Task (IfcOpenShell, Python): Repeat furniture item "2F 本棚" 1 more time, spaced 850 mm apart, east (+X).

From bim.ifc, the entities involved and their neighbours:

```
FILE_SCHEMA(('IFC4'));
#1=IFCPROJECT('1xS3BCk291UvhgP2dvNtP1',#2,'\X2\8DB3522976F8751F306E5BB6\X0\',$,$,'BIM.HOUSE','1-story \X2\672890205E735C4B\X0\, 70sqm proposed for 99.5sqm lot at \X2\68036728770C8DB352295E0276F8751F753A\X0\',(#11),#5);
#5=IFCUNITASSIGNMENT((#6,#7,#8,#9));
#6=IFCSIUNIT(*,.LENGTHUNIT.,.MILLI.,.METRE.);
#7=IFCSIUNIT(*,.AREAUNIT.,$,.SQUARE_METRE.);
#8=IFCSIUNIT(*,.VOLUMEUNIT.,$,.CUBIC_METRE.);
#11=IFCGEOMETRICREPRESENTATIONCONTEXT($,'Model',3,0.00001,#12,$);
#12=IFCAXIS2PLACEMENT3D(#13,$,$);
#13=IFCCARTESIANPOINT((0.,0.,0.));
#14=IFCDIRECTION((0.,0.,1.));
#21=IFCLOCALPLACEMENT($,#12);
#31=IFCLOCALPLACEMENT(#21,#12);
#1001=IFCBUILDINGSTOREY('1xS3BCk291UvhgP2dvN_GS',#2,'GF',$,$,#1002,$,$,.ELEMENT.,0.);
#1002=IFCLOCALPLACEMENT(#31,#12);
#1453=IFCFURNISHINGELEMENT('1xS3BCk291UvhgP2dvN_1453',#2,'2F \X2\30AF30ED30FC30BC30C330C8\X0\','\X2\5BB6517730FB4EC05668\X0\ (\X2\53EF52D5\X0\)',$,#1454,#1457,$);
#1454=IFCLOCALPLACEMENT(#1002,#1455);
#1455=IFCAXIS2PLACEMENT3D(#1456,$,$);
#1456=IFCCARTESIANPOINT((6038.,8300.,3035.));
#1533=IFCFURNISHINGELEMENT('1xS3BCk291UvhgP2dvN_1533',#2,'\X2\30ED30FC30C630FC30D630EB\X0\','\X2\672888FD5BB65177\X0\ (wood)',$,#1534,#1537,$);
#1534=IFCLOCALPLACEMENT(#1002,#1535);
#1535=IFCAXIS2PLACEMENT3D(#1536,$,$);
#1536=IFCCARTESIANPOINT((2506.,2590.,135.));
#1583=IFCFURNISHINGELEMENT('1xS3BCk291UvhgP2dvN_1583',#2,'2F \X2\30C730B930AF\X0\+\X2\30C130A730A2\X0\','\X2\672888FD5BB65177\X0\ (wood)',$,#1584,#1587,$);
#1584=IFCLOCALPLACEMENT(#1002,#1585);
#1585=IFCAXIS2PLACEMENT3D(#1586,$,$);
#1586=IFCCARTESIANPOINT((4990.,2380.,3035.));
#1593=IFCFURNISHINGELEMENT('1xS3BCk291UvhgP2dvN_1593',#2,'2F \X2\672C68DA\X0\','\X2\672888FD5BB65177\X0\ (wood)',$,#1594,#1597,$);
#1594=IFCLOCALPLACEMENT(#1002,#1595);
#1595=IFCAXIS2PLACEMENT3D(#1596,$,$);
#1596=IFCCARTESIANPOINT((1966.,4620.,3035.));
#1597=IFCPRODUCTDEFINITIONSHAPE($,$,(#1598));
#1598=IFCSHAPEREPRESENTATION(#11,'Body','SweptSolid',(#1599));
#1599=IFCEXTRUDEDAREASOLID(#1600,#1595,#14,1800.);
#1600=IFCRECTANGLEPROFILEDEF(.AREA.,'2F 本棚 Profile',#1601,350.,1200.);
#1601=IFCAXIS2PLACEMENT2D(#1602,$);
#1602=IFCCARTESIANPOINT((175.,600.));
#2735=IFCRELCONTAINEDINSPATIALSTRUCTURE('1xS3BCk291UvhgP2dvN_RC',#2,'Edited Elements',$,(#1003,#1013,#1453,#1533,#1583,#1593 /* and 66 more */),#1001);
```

```python
import numpy as np
import ifcopenshell
import ifcopenshell.api.geometry
import ifcopenshell.api.root
import ifcopenshell.util.element
import ifcopenshell.util.placement
import ifcopenshell.util.unit

model = ifcopenshell.open("bim.ifc")
unit_scale = ifcopenshell.util.unit.calculate_unit_scale(model)


def reuse_history(source, copy):
    """copy_class also copies each property set's owner history, people and application; keep the originals."""
    for rel in copy.IsDefinedBy:
        if rel.is_a("IfcRelDefinesByProperties") and (history := rel.RelatingPropertyDefinition.OwnerHistory):
            rel.RelatingPropertyDefinition.OwnerHistory = source.OwnerHistory
            ifcopenshell.util.element.remove_deep2(model, history)


source = model.by_guid("1xS3BCk291UvhgP2dvN_1593")
base = ifcopenshell.util.placement.get_local_placement(source.ObjectPlacement)
step = np.array([1.0, 0.0, 0.0]) * 0.85 / unit_scale

for i in range(1, 2):
    copy = ifcopenshell.api.root.copy_class(model, product=source)
    copy.Representation = ifcopenshell.util.element.copy_deep(
        model, source.Representation, exclude=["IfcGeometricRepresentationContext", "IfcRepresentationMap"]
    )
    reuse_history(source, copy)
    matrix = base.copy()
    matrix[:3, 3] += i * step
    print("added at", matrix[:3, 3].round(3) + 0.0)
    ifcopenshell.api.geometry.edit_object_placement(model, product=copy, matrix=matrix, is_si=False)

model.write("bim_updated.ifc")
```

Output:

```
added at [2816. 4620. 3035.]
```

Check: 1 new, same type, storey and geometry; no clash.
